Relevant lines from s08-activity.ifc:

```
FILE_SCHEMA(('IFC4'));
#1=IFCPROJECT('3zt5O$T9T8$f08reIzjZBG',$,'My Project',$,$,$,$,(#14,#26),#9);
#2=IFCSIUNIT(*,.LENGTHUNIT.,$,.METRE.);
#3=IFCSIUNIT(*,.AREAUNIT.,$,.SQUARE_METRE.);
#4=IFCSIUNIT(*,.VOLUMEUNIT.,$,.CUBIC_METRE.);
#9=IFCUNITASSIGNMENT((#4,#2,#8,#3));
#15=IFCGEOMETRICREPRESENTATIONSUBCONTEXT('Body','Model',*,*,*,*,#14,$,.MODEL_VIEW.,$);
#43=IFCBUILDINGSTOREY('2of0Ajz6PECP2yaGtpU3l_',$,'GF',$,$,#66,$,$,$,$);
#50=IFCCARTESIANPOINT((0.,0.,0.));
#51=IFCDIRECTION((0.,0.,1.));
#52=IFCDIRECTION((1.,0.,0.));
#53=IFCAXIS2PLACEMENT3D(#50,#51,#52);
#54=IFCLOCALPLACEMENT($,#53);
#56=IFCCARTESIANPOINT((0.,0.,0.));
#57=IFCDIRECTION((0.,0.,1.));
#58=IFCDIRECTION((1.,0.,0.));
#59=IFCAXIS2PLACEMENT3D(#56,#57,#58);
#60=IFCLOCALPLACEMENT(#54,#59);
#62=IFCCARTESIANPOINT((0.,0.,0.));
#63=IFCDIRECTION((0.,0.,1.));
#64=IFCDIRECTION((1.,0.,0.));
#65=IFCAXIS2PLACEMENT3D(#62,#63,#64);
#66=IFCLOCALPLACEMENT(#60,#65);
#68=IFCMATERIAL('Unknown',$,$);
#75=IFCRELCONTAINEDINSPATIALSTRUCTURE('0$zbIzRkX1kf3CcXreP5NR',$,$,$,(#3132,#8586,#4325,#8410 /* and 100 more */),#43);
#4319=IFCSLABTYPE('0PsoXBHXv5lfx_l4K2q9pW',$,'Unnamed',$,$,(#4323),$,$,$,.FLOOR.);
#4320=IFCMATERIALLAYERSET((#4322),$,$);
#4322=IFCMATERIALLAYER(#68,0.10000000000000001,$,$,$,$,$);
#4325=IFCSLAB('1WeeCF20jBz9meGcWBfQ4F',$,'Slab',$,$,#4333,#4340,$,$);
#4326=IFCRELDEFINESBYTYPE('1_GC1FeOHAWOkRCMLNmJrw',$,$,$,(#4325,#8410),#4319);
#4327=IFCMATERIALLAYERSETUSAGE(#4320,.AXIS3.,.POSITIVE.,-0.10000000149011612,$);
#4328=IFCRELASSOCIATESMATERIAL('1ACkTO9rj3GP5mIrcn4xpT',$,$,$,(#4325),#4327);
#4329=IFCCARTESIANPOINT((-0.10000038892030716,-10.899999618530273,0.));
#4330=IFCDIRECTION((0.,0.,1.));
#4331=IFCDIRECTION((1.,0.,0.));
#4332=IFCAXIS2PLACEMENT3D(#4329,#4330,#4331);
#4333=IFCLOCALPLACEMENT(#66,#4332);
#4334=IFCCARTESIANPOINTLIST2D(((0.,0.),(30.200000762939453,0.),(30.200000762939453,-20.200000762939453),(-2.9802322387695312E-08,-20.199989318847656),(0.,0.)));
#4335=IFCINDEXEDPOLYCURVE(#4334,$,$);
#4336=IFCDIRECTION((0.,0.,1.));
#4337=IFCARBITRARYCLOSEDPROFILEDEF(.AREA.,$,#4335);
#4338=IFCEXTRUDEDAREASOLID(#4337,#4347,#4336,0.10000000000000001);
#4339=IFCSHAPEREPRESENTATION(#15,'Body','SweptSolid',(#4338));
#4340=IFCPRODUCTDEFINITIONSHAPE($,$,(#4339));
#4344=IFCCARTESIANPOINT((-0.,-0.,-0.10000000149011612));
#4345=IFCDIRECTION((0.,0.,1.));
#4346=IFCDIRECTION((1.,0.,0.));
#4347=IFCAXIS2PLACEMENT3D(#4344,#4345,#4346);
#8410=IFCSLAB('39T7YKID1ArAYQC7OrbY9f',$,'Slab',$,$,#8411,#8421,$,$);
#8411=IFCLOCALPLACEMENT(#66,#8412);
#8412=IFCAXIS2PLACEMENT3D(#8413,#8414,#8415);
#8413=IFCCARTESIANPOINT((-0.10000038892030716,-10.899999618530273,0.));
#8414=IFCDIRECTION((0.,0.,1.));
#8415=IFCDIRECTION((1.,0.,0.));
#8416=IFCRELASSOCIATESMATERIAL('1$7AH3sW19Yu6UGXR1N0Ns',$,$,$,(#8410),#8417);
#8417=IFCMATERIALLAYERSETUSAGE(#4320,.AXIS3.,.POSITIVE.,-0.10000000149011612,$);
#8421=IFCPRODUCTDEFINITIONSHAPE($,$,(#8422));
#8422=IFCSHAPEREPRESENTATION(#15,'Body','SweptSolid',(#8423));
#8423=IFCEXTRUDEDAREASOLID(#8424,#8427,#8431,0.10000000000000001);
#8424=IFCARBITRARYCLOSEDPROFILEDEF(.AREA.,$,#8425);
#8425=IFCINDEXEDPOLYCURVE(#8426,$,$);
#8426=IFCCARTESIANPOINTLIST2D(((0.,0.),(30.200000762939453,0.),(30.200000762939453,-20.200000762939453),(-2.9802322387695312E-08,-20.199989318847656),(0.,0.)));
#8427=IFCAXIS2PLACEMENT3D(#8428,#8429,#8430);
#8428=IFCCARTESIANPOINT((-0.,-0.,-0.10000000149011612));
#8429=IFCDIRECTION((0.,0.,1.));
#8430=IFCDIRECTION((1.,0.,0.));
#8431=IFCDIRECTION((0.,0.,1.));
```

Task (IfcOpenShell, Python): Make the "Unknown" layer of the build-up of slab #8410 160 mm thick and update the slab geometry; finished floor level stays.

```python
import ifcopenshell
import ifcopenshell.util.element
import ifcopenshell.util.representation

model = ifcopenshell.open("s08-activity.ifc")

layer_set = model.by_id(4320)
layer = next(l for l in layer_set.MaterialLayers if l.Material and l.Material.Name == "Unknown")
change = 0.16 - layer.LayerThickness
layer.LayerThickness += change

# The layer set is shared, so every slab that uses it gets the new thickness.
slabs = [e for e in ifcopenshell.util.element.get_elements_by_material(model, layer_set) if e.is_a("IfcSlab")]
for slab in sorted(slabs, key=lambda e: e.id()):
    body = ifcopenshell.util.representation.get_representation(slab, "Model", "Body")
    solid = body.Items[0]
    old_depth = solid.Depth
    solid.Depth += change
    # Extruded upwards: lower the start of the extrusion so the top stays.
    x, y, z = solid.Position.Location.Coordinates
    solid.Position.Location = model.createIfcCartesianPoint((x, y, z - change))
    print(slab.id(), f"{old_depth:g} -> {solid.Depth:g}")

# The layers are counted up from the underside, which has moved.
for usage in {ifcopenshell.util.element.get_material(slab) for slab in slabs}:
    usage.OffsetFromReferenceLine -= change

model.write("s08-activity_edited.ifc")
```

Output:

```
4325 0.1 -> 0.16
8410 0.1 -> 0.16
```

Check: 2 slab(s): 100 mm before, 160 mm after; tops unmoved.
